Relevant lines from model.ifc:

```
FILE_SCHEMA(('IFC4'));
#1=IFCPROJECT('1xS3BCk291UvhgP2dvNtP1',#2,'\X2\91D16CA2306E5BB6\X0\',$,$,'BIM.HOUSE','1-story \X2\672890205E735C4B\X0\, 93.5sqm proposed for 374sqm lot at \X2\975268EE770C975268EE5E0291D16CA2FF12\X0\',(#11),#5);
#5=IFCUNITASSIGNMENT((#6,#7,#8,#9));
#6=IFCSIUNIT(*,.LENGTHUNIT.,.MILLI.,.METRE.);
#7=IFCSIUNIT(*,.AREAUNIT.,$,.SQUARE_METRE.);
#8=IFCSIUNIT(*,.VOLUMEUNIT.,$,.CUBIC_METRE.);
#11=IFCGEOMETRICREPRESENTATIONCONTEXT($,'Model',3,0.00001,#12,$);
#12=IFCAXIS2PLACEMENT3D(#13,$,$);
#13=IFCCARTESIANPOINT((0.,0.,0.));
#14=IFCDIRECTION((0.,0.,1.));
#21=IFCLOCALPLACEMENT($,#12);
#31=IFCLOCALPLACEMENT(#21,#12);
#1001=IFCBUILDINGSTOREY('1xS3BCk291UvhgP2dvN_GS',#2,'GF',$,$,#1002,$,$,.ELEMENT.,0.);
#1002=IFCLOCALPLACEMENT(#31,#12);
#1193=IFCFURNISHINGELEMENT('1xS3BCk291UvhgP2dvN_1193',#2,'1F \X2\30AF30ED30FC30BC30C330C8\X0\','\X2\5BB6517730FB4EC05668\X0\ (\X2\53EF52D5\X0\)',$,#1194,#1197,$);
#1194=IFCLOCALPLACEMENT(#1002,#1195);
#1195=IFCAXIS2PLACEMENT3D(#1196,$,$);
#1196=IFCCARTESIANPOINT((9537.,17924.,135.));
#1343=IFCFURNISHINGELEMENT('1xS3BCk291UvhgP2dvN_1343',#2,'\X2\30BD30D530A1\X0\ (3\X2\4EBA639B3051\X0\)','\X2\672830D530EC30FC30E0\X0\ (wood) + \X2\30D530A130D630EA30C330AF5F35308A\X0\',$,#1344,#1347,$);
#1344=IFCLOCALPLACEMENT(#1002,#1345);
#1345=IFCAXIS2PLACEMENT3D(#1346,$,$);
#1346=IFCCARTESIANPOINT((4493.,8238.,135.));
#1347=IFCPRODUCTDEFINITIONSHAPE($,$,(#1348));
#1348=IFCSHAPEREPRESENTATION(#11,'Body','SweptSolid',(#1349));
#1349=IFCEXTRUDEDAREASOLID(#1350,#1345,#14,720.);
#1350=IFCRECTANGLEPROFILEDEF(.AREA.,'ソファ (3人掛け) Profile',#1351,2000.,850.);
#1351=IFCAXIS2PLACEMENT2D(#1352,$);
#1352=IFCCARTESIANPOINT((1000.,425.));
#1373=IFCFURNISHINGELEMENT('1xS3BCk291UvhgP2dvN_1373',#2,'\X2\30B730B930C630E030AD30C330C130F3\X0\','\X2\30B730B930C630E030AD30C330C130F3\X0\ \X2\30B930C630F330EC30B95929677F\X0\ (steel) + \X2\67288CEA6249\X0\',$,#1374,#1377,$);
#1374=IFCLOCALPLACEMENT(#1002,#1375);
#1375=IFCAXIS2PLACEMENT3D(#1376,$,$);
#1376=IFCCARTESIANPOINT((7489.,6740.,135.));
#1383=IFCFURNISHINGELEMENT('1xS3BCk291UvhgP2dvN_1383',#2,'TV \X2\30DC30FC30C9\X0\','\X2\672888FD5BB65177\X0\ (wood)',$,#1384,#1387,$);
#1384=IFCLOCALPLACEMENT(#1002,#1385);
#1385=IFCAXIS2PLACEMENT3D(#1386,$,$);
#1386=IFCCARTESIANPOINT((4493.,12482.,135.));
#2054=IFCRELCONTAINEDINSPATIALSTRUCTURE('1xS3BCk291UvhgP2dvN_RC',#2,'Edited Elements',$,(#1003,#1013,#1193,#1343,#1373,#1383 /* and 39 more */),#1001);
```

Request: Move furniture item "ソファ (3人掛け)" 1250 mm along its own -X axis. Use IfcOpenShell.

```python
import ifcopenshell
import ifcopenshell.api.geometry
import ifcopenshell.util.placement
import ifcopenshell.util.unit

model = ifcopenshell.open("model.ifc")
unit_scale = ifcopenshell.util.unit.calculate_unit_scale(model)

item = model.by_guid("1xS3BCk291UvhgP2dvN_1343")
matrix = ifcopenshell.util.placement.get_local_placement(item.ObjectPlacement)
matrix[:3, 3] -= matrix[:3, 0] * 1.25 / unit_scale
ifcopenshell.api.geometry.edit_object_placement(model, product=item, matrix=matrix, is_si=False)

print(ifcopenshell.util.placement.get_local_placement(item.ObjectPlacement).round(3) + 0.0)

model.write("model_rev.ifc")
```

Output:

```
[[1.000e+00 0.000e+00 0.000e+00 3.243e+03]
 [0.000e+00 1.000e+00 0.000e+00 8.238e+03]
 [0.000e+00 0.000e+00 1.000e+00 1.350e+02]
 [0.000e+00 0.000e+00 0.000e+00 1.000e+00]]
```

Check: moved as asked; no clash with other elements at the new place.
